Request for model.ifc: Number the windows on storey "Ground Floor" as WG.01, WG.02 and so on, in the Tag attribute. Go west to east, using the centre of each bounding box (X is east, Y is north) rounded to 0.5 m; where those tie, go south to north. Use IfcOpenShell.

First a look at what the model holds.

```python
import ifcopenshell
import ifcopenshell.util.element
import ifcopenshell.util.placement

model = ifcopenshell.open("model.ifc")
print(model.schema)
storey = next(s for s in model.by_type("IfcBuildingStorey") if s.Name == "Ground Floor")
windows = [e for e in ifcopenshell.util.element.get_decomposition(storey) if e.is_a("IfcWindow")]
for e in sorted(windows, key=lambda e: e.id()):
    origin = ifcopenshell.util.placement.get_local_placement(e.ObjectPlacement)[:3, 3]
    print(e.id(), e.Tag, e.Name, origin.round(2) + 0.0, sep=" | ")
```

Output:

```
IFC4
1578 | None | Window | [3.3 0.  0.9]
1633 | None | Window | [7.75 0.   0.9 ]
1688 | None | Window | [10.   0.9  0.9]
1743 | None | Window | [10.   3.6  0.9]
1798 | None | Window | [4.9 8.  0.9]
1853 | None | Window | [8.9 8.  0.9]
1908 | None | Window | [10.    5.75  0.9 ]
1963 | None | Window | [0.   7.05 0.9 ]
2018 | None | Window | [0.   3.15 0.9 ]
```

```python
import ifcopenshell
import ifcopenshell.geom
import ifcopenshell.util.element
import ifcopenshell.util.shape

model = ifcopenshell.open("model.ifc")
settings = ifcopenshell.geom.settings()
settings.set("use-world-coords", True)


def centre(element):
    shape = ifcopenshell.geom.create_shape(settings, element)
    return ifcopenshell.util.shape.get_bbox_centroid(shape.geometry)


storey = next(s for s in model.by_type("IfcBuildingStorey") if s.Name == "Ground Floor")
windows = [e for e in ifcopenshell.util.element.get_decomposition(storey) if e.is_a("IfcWindow")]

# Insertion points can sit at a corner or the storey origin, so sort by the geometry (in metres).
centres = {e: centre(e) for e in windows}
windows.sort(key=lambda e: (round(centres[e][0] / 0.5), centres[e][1]))

for i, e in enumerate(windows, start=1):
    number = f"WG.{i:02d}"
    e.Tag = number
    print(e.id(), number)

model.write("model_v2.ifc")
```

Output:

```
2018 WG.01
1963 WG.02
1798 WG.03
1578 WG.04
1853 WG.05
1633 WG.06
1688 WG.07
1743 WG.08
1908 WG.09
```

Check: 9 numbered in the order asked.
